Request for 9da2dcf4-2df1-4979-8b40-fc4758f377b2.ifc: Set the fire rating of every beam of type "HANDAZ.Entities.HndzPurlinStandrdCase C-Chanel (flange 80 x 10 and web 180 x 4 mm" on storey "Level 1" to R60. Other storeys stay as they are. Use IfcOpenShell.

First a look at what the model holds.

```python
import ifcopenshell
import ifcopenshell.util.element

model = ifcopenshell.open("9da2dcf4-2df1-4979-8b40-fc4758f377b2.ifc")
print(model.schema)
storey = next(s for s in model.by_type("IfcBuildingStorey") if s.Name == "Level 1")
beams = [e for e in ifcopenshell.util.element.get_decomposition(storey) if e.is_a("IfcBeam")]
seen = {}
for e in beams:
    element_type = ifcopenshell.util.element.get_type(e)
    key = (element_type.Name if element_type != e and element_type else None, ifcopenshell.util.element.get_pset(e, "Pset_BeamCommon", "FireRating"))
    seen[key] = seen.get(key, 0) + 1
for (name, value), count in sorted(seen.items(), key=str):
    print(count, "x", name, "|", value)
```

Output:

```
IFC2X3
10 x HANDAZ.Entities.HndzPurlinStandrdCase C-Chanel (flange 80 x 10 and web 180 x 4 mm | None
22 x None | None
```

```python
import ifcopenshell
import ifcopenshell.api.pset
import ifcopenshell.util.element

model = ifcopenshell.open("9da2dcf4-2df1-4979-8b40-fc4758f377b2.ifc")

storey = next(s for s in model.by_type("IfcBuildingStorey") if s.Name == "Level 1")
beams = [e for e in ifcopenshell.util.element.get_decomposition(storey) if e.is_a("IfcBeam")]

count = 0
for e in beams:
    element_type = ifcopenshell.util.element.get_type(e)
    if element_type in (None, e) or element_type.Name != "HANDAZ.Entities.HndzPurlinStandrdCase C-Chanel (flange 80 x 10 and web 180 x 4 mm":
        continue
    # add_pset returns the element's existing set when there is one.
    pset = ifcopenshell.api.pset.add_pset(model, product=e, name="Pset_BeamCommon")
    ifcopenshell.api.pset.edit_pset(model, pset=pset, properties={"FireRating": "R60"})
    count += 1

print(count, "beams updated")

model.write("9da2dcf4-2df1-4979-8b40-fc4758f377b2_updated.ifc")
```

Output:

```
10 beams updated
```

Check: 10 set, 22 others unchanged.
